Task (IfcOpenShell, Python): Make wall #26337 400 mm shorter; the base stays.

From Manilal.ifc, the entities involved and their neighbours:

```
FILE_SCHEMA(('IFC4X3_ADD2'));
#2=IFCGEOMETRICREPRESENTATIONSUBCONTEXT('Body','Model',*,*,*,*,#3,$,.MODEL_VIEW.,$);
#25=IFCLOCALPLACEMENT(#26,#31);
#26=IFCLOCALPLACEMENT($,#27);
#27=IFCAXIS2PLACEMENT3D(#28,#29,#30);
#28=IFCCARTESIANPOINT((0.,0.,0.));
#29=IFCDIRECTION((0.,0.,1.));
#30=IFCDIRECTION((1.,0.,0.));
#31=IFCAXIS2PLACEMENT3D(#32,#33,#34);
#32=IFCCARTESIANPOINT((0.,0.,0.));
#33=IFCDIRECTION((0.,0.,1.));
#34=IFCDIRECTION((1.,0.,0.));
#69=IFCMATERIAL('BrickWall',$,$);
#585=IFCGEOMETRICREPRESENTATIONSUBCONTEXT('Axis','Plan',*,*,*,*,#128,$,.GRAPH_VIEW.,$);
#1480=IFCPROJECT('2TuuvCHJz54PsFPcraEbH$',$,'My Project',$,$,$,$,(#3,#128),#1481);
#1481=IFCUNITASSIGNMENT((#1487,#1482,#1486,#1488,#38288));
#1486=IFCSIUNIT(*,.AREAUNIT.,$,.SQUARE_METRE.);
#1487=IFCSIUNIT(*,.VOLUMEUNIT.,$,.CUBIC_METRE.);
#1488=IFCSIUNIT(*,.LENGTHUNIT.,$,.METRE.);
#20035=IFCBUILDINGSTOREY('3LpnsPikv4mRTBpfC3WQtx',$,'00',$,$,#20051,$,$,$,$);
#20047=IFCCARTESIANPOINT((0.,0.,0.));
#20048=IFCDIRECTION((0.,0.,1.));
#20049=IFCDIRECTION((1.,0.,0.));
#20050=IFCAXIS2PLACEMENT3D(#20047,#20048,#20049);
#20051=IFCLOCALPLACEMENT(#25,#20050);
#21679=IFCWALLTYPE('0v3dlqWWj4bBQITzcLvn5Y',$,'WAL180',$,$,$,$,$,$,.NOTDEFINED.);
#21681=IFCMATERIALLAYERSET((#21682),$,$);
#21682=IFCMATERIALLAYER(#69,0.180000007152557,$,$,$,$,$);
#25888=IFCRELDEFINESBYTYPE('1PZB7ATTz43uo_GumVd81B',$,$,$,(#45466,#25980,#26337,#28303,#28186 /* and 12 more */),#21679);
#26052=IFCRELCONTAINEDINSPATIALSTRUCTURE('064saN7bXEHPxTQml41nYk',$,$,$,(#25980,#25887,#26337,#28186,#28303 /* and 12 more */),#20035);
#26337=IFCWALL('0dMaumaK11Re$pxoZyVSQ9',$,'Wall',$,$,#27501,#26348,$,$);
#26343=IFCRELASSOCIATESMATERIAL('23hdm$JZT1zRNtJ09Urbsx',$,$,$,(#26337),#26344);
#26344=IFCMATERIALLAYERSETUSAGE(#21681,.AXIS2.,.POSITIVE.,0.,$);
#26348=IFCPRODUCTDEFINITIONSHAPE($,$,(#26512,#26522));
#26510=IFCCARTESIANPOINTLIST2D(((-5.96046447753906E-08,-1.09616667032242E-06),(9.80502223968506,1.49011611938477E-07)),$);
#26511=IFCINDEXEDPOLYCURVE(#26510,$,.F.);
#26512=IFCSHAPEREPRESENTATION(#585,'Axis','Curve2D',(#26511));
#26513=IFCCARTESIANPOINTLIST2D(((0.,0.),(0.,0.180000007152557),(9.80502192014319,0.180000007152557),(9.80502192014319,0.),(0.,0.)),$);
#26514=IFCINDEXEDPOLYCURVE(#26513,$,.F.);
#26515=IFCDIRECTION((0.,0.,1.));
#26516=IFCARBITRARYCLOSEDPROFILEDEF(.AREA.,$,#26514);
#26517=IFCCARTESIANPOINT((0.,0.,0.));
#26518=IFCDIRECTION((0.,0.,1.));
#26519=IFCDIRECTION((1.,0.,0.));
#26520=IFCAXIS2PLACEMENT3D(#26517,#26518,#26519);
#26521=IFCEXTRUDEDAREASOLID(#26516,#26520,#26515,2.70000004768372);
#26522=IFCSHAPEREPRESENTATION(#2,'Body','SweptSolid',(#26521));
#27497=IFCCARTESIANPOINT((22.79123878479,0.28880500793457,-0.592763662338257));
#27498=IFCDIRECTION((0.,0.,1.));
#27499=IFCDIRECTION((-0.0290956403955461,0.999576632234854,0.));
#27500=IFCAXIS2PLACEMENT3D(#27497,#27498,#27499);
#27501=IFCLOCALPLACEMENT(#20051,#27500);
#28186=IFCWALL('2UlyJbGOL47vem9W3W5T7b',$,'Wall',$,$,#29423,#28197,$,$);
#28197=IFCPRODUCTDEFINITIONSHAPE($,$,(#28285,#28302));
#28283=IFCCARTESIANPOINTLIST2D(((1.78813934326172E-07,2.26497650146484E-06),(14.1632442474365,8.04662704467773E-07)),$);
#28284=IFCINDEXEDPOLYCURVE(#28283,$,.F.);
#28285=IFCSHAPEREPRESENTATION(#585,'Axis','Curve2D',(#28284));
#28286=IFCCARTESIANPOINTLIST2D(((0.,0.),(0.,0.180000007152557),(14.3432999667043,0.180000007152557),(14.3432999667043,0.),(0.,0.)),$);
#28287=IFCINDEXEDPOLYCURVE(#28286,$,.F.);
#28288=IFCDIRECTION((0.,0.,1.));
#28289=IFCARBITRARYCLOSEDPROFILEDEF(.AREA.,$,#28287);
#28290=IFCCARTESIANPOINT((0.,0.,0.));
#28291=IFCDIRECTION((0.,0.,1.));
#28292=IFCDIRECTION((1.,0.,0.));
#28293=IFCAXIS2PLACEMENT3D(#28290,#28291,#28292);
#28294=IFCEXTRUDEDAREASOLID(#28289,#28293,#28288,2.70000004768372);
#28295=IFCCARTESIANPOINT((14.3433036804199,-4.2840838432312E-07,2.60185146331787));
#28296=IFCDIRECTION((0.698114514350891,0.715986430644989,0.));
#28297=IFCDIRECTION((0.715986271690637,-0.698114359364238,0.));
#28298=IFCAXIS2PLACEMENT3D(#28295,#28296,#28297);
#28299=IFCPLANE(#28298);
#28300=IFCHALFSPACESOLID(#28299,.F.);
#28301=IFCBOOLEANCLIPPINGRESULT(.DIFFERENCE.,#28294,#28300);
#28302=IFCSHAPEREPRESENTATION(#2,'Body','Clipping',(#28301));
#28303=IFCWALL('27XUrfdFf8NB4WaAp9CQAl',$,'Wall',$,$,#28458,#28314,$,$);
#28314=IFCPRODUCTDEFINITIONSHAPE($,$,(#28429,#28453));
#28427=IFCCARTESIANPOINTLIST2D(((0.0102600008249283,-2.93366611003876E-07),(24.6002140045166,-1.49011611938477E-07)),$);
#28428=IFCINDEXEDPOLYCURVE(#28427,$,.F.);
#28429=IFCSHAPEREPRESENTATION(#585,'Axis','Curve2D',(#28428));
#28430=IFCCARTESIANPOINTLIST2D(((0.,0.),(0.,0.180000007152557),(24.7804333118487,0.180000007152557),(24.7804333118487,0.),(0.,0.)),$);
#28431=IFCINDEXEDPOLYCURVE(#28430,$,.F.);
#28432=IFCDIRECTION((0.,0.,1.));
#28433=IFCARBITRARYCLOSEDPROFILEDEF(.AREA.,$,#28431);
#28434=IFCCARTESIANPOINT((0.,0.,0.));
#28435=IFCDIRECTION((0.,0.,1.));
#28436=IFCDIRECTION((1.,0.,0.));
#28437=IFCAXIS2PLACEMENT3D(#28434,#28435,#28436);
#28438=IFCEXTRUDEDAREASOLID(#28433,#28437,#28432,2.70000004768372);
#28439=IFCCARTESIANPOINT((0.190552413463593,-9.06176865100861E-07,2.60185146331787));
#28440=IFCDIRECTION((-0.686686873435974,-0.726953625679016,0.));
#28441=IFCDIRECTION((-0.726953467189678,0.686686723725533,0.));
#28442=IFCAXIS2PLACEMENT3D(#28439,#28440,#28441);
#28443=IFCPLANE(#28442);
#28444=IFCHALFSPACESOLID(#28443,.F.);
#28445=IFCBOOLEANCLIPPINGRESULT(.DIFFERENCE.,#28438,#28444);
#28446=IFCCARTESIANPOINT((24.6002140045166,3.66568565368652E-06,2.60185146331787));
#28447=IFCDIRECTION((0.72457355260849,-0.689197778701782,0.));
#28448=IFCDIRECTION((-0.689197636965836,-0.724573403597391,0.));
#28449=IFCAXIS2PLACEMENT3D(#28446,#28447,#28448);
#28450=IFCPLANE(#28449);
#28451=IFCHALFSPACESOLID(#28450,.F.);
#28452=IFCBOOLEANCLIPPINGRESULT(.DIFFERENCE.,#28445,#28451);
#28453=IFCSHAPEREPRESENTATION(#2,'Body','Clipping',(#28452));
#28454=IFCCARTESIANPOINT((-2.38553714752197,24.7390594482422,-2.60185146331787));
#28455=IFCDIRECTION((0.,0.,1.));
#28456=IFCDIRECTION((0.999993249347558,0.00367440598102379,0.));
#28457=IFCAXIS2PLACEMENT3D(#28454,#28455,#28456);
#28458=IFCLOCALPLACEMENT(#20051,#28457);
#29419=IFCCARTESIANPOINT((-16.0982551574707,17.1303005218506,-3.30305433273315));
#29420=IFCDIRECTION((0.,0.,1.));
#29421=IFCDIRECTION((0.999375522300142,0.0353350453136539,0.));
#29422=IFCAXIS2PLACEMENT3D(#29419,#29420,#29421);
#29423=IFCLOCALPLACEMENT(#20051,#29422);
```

```python
import ifcopenshell
import ifcopenshell.geom
import ifcopenshell.util.representation
import ifcopenshell.util.shape
import ifcopenshell.util.unit

model = ifcopenshell.open("Manilal.ifc")
unit_scale = ifcopenshell.util.unit.calculate_unit_scale(model)
settings = ifcopenshell.geom.settings()


def volume(element):
    """Net volume in cubic metres, openings subtracted."""
    shape = ifcopenshell.geom.create_shape(settings, element)
    return ifcopenshell.util.shape.get_volume(shape.geometry)


wall = model.by_guid("0dMaumaK11Re$pxoZyVSQ9")
before = volume(wall)

body = ifcopenshell.util.representation.get_representation(wall, "Model", "Body")
solid = body.Items[0]
old_height = solid.Depth
solid.Depth -= 0.4 / unit_scale
after = volume(wall)

print(f"height {old_height:g} -> {solid.Depth:g}, volume {before:.3f} -> {after:.3f} m3")

model.write("Manilal_v2.ifc")
```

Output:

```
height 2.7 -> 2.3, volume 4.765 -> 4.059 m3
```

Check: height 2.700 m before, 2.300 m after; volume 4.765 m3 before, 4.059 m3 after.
